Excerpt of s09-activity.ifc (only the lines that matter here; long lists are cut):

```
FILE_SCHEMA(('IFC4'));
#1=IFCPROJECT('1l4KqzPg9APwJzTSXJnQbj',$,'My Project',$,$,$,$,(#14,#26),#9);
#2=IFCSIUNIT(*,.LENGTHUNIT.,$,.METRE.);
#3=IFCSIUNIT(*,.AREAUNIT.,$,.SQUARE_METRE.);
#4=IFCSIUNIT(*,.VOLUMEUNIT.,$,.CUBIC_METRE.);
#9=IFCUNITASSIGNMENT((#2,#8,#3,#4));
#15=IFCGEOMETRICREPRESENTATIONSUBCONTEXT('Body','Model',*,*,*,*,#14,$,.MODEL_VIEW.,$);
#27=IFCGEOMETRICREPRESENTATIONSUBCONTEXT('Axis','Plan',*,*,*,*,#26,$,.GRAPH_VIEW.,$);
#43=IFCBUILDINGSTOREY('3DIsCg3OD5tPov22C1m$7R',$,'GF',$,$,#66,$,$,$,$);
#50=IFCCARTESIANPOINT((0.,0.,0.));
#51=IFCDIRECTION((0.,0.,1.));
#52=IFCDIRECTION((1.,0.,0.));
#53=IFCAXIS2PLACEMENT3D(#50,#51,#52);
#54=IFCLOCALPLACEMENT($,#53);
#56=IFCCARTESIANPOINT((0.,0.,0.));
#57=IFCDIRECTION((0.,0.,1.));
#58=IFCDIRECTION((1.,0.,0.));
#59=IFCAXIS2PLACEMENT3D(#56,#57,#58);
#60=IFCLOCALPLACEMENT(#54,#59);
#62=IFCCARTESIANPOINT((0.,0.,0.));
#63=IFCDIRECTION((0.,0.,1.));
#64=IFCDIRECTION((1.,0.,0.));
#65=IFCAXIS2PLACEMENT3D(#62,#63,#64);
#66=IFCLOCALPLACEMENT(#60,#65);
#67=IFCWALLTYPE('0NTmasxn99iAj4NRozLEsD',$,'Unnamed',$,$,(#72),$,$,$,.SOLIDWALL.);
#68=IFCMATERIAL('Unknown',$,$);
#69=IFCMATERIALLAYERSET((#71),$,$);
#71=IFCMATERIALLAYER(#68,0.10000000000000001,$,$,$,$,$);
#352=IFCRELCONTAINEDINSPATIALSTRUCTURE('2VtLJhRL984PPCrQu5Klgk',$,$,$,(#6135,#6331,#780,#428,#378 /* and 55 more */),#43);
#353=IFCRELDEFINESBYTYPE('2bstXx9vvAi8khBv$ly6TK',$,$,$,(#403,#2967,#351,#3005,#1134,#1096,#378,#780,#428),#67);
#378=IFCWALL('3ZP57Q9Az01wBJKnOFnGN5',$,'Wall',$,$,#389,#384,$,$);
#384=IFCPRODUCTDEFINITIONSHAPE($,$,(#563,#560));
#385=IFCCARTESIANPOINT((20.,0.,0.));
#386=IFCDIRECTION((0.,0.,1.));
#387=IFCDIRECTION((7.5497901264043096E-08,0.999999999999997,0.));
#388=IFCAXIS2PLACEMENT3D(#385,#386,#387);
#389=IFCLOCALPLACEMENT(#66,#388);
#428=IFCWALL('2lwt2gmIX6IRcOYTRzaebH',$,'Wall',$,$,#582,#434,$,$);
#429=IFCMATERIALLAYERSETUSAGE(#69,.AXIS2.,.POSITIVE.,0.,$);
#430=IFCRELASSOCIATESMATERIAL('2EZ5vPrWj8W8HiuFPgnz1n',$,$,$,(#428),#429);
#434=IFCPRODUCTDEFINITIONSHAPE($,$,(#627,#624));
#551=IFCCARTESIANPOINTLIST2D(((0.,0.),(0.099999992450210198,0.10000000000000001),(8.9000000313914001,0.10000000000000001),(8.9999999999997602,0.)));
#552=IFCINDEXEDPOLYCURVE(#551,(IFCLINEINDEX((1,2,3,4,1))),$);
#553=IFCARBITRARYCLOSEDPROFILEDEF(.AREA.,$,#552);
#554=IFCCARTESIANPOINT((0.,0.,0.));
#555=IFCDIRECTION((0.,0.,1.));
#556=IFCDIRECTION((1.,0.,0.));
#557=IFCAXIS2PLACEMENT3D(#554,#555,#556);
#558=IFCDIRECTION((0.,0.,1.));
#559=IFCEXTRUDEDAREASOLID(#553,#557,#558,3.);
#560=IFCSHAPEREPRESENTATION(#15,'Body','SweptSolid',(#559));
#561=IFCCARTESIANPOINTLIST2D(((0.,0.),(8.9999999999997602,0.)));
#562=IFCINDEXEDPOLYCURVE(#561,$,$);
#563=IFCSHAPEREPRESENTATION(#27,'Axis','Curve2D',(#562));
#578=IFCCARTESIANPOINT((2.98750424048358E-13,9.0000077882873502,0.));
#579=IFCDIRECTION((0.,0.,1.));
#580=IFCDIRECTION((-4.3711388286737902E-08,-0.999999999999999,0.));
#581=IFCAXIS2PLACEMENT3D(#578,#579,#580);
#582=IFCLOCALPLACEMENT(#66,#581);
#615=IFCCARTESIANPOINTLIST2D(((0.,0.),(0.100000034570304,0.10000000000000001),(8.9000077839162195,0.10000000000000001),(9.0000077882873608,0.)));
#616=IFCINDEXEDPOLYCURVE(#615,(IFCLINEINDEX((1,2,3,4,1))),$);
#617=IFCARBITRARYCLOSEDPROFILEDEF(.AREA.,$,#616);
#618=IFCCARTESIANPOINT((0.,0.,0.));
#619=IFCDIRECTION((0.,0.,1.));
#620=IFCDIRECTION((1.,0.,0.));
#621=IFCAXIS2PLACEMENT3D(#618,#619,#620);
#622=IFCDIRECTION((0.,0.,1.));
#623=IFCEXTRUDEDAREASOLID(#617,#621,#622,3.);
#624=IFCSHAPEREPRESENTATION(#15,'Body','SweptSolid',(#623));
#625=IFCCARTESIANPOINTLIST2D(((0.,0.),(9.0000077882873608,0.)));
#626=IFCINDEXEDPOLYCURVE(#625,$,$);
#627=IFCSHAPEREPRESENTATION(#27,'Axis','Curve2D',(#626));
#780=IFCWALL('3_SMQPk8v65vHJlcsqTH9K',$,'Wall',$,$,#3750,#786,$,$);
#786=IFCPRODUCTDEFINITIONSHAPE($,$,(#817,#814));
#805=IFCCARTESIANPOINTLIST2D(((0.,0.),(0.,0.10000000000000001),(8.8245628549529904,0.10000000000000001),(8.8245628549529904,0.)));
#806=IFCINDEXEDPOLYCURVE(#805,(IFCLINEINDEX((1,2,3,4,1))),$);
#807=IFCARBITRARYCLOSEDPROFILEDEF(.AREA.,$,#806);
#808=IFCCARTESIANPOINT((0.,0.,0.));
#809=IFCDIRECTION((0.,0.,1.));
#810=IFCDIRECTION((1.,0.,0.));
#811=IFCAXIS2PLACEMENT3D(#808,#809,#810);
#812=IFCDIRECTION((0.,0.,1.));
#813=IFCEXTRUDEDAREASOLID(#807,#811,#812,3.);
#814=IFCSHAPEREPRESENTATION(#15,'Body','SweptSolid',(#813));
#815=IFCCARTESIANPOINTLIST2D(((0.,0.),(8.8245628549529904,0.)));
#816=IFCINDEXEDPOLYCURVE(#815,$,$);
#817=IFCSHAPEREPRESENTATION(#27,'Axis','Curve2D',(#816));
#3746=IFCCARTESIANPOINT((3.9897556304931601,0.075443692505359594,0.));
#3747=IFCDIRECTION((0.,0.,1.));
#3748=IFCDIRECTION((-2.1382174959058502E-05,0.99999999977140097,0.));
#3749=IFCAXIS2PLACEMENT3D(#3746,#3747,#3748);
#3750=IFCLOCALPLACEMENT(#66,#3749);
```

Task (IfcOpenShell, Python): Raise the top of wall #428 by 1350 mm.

```python
import ifcopenshell
import ifcopenshell.geom
import ifcopenshell.util.representation
import ifcopenshell.util.shape

model = ifcopenshell.open("s09-activity.ifc")
settings = ifcopenshell.geom.settings()


def volume(element):
    """Net volume in cubic metres, openings subtracted."""
    shape = ifcopenshell.geom.create_shape(settings, element)
    return ifcopenshell.util.shape.get_volume(shape.geometry)


wall = model.by_guid("2lwt2gmIX6IRcOYTRzaebH")
before = volume(wall)

body = ifcopenshell.util.representation.get_representation(wall, "Model", "Body")
solid = body.Items[0]
old_height = solid.Depth
solid.Depth += 1.35
after = volume(wall)

print(f"height {old_height:g} -> {solid.Depth:g}, volume {before:.3f} -> {after:.3f} m3")

model.write("s09-activity-out.ifc")
```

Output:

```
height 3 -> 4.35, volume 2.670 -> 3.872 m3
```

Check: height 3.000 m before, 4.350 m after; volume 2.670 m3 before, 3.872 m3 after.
